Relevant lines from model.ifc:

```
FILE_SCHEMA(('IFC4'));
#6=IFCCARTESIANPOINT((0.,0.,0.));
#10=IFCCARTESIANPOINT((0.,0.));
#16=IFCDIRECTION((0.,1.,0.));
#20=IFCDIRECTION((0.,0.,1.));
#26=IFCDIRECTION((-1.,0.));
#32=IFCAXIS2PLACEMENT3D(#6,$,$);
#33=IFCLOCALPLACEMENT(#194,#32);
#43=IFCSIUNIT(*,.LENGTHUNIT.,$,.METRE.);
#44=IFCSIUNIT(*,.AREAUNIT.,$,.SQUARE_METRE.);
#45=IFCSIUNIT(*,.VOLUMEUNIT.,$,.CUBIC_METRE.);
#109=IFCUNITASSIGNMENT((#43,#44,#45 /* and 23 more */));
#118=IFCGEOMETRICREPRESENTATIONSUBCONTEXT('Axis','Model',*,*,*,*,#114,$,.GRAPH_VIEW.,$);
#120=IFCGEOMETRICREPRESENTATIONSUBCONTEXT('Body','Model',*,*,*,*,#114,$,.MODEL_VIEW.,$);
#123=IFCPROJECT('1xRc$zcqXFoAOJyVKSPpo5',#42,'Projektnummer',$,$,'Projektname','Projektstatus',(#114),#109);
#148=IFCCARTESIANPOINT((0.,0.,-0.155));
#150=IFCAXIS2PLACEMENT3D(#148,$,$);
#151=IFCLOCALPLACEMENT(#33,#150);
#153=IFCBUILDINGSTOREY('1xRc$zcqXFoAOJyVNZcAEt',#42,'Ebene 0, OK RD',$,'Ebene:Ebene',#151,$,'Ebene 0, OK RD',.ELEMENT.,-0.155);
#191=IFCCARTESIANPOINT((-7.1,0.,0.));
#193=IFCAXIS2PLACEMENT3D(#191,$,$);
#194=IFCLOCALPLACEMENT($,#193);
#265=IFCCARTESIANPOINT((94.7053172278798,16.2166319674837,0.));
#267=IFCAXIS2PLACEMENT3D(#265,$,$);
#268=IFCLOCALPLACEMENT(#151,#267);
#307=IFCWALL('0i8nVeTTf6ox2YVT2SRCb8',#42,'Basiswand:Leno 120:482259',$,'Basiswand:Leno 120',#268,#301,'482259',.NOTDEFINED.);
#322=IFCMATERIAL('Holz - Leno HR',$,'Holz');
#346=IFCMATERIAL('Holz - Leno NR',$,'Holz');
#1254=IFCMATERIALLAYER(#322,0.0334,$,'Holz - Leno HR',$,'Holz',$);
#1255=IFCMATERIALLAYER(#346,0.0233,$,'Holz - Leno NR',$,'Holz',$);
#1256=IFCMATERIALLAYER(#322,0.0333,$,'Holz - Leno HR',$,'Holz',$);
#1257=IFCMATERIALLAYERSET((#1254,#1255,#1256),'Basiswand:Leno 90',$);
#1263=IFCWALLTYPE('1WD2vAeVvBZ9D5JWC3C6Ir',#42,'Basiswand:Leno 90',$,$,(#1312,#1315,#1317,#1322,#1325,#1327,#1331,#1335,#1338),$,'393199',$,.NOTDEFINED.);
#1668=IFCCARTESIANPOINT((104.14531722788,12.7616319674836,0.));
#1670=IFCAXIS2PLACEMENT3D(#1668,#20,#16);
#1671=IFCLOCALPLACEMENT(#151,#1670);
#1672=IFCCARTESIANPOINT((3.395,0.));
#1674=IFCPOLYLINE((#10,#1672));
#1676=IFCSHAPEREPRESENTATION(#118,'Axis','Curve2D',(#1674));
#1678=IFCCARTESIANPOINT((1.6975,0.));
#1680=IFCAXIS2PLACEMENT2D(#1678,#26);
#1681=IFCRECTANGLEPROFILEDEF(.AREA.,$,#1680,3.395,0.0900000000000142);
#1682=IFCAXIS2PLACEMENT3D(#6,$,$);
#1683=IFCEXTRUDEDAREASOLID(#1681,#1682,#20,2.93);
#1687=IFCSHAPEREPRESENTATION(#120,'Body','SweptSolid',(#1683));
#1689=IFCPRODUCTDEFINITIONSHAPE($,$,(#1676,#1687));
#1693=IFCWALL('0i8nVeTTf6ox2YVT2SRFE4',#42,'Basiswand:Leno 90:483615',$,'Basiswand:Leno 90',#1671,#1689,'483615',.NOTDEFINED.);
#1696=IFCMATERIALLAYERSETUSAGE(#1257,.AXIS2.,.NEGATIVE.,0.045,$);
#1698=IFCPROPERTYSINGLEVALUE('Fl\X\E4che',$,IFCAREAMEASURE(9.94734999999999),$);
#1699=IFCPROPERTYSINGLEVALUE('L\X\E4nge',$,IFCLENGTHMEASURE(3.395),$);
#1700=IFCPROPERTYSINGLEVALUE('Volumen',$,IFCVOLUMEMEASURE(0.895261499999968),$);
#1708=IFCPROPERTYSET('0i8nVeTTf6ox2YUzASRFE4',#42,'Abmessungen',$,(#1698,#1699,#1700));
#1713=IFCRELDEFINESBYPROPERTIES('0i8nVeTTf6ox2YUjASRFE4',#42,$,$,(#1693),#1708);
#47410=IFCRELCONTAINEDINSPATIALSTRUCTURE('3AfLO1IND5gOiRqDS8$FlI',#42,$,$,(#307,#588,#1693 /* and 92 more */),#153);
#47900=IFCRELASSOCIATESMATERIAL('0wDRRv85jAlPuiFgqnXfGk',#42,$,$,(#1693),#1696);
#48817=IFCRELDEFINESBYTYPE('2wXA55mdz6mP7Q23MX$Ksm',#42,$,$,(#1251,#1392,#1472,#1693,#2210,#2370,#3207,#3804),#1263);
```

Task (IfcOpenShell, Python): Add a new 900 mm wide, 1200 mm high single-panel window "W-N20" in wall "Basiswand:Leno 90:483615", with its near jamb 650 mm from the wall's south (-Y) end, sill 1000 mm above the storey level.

```python
import numpy as np
import ifcopenshell
import ifcopenshell.api.feature
import ifcopenshell.api.geometry
import ifcopenshell.api.pset
import ifcopenshell.api.root
import ifcopenshell.api.spatial
import ifcopenshell.geom
import ifcopenshell.util.element
import ifcopenshell.util.placement
import ifcopenshell.util.representation
import ifcopenshell.util.shape
import ifcopenshell.util.unit

model = ifcopenshell.open("model.ifc")
unit_scale = ifcopenshell.util.unit.calculate_unit_scale(model)
area_scale = ifcopenshell.util.unit.calculate_unit_scale(model, "AREAUNIT")
volume_scale = ifcopenshell.util.unit.calculate_unit_scale(model, "VOLUMEUNIT")
settings = ifcopenshell.geom.settings()


def volume(element):
    """Net volume in cubic metres, openings subtracted."""
    shape = ifcopenshell.geom.create_shape(settings, element)
    return ifcopenshell.util.shape.get_volume(shape.geometry)


wall = model.by_guid("0i8nVeTTf6ox2YVT2SRFE4")
storey = ifcopenshell.util.element.get_container(wall, ifc_class="IfcBuildingStorey")
context = ifcopenshell.util.representation.get_context(model, "Model", "Body", "MODEL_VIEW")
before = volume(wall)

width, height, from_end, sill = 0.9, 1.2, 0.65, 1  # metres

# The wall runs along its own X axis, and the end named is its -X end.
wall_shape = ifcopenshell.geom.create_shape(settings, wall)
x, y, z = ifcopenshell.util.shape.get_vertices(wall_shape.geometry).T
start = x.min() + from_end
face, thickness = float(y.min()), float(y.max() - y.min())
wall_matrix = ifcopenshell.util.placement.get_local_placement(wall.ObjectPlacement)
level = ifcopenshell.util.placement.get_local_placement(storey.ObjectPlacement)[2, 3]


def in_wall(x, y):
    """Placement at x, y metres in the wall's axes, at sill height."""
    matrix = wall_matrix.copy()
    matrix[:, 3] = wall_matrix @ np.array([x / unit_scale, y / unit_scale, 0.0, 1.0])
    matrix[2, 3] = level + sill / unit_scale
    return matrix


# Opening: a box that overshoots both wall faces by 50 mm.
opening = ifcopenshell.api.root.create_entity(model, ifc_class="IfcOpeningElement", predefined_type="OPENING")
box = ifcopenshell.api.geometry.add_wall_representation(
    model, context=context, length=width, height=height, thickness=thickness + 0.1
)
ifcopenshell.api.geometry.assign_representation(model, product=opening, representation=box)
ifcopenshell.api.geometry.edit_object_placement(model, product=opening, matrix=in_wall(start, face - 0.05), is_si=False)
ifcopenshell.api.feature.add_feature(model, feature=opening, element=wall)

window = ifcopenshell.api.root.create_entity(model, ifc_class="IfcWindow", name="W-N20", predefined_type="WINDOW")
window.OverallWidth, window.OverallHeight = width / unit_scale, height / unit_scale
window.PartitioningType = "SINGLE_PANEL"
body = ifcopenshell.api.geometry.add_window_representation(
    model,
    context=context,
    overall_width=window.OverallWidth,
    overall_height=window.OverallHeight,
    partition_type="SINGLE_PANEL",
)
ifcopenshell.api.geometry.assign_representation(model, product=window, representation=body)
ifcopenshell.api.spatial.assign_container(model, products=[window], relating_structure=storey)
ifcopenshell.api.feature.add_filling(model, opening=opening, element=window)

# Centre the window in the wall's thickness.
ifcopenshell.api.geometry.edit_object_placement(model, product=window, matrix=in_wall(start, face), is_si=False)
window_shape = ifcopenshell.geom.create_shape(settings, window)
depth = ifcopenshell.util.shape.get_vertices(window_shape.geometry)[:, 1]
offset = face + thickness / 2 - (depth.min() + depth.max()) / 2
ifcopenshell.api.geometry.edit_object_placement(model, product=window, matrix=in_wall(start, offset), is_si=False)

after = volume(wall)

# Update the wall's stored quantities.
pset = model.by_id(ifcopenshell.util.element.get_pset(wall, "Abmessungen", should_inherit=False)["id"])
ifcopenshell.api.pset.edit_pset(model, pset=pset, properties={
    "Fläche": model.create_entity("IfcAreaMeasure", after / thickness / area_scale),
    "Volumen": model.create_entity("IfcVolumeMeasure", after / volume_scale),
})

print(f"wall volume {before:.3f} -> {after:.3f} m3")

model.write("model_rev.ifc")
```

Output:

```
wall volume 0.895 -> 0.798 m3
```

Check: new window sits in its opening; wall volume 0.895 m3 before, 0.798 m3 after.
